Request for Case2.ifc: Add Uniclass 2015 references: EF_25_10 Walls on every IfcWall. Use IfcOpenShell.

First a look at what the model holds.

```python
import ifcopenshell

model = ifcopenshell.open("Case2.ifc")
print(model.schema)
print("classifications:", [c.Name for c in model.by_type("IfcClassification")])
for ifc_class in ("IfcDoor", "IfcRoof", "IfcStair", "IfcWall", "IfcWindow"):
    print(ifc_class, len(model.by_type(ifc_class)))
```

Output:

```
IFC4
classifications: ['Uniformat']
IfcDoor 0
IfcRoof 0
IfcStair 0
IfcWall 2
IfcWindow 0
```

```python
import ifcopenshell
import ifcopenshell.api.classification

model = ifcopenshell.open("Case2.ifc")

system = ifcopenshell.api.classification.add_classification(model, classification="Uniclass 2015")

codes = {
    "IfcWall": ("EF_25_10", "Walls"),
}
for ifc_class, (code, name) in codes.items():
    products = model.by_type(ifc_class)
    ifcopenshell.api.classification.add_reference(
        model, products=products, classification=system, identification=code, name=name
    )
    print(code, len(products))

model.write("Case2_updated.ifc")
```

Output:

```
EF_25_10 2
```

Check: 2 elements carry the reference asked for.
